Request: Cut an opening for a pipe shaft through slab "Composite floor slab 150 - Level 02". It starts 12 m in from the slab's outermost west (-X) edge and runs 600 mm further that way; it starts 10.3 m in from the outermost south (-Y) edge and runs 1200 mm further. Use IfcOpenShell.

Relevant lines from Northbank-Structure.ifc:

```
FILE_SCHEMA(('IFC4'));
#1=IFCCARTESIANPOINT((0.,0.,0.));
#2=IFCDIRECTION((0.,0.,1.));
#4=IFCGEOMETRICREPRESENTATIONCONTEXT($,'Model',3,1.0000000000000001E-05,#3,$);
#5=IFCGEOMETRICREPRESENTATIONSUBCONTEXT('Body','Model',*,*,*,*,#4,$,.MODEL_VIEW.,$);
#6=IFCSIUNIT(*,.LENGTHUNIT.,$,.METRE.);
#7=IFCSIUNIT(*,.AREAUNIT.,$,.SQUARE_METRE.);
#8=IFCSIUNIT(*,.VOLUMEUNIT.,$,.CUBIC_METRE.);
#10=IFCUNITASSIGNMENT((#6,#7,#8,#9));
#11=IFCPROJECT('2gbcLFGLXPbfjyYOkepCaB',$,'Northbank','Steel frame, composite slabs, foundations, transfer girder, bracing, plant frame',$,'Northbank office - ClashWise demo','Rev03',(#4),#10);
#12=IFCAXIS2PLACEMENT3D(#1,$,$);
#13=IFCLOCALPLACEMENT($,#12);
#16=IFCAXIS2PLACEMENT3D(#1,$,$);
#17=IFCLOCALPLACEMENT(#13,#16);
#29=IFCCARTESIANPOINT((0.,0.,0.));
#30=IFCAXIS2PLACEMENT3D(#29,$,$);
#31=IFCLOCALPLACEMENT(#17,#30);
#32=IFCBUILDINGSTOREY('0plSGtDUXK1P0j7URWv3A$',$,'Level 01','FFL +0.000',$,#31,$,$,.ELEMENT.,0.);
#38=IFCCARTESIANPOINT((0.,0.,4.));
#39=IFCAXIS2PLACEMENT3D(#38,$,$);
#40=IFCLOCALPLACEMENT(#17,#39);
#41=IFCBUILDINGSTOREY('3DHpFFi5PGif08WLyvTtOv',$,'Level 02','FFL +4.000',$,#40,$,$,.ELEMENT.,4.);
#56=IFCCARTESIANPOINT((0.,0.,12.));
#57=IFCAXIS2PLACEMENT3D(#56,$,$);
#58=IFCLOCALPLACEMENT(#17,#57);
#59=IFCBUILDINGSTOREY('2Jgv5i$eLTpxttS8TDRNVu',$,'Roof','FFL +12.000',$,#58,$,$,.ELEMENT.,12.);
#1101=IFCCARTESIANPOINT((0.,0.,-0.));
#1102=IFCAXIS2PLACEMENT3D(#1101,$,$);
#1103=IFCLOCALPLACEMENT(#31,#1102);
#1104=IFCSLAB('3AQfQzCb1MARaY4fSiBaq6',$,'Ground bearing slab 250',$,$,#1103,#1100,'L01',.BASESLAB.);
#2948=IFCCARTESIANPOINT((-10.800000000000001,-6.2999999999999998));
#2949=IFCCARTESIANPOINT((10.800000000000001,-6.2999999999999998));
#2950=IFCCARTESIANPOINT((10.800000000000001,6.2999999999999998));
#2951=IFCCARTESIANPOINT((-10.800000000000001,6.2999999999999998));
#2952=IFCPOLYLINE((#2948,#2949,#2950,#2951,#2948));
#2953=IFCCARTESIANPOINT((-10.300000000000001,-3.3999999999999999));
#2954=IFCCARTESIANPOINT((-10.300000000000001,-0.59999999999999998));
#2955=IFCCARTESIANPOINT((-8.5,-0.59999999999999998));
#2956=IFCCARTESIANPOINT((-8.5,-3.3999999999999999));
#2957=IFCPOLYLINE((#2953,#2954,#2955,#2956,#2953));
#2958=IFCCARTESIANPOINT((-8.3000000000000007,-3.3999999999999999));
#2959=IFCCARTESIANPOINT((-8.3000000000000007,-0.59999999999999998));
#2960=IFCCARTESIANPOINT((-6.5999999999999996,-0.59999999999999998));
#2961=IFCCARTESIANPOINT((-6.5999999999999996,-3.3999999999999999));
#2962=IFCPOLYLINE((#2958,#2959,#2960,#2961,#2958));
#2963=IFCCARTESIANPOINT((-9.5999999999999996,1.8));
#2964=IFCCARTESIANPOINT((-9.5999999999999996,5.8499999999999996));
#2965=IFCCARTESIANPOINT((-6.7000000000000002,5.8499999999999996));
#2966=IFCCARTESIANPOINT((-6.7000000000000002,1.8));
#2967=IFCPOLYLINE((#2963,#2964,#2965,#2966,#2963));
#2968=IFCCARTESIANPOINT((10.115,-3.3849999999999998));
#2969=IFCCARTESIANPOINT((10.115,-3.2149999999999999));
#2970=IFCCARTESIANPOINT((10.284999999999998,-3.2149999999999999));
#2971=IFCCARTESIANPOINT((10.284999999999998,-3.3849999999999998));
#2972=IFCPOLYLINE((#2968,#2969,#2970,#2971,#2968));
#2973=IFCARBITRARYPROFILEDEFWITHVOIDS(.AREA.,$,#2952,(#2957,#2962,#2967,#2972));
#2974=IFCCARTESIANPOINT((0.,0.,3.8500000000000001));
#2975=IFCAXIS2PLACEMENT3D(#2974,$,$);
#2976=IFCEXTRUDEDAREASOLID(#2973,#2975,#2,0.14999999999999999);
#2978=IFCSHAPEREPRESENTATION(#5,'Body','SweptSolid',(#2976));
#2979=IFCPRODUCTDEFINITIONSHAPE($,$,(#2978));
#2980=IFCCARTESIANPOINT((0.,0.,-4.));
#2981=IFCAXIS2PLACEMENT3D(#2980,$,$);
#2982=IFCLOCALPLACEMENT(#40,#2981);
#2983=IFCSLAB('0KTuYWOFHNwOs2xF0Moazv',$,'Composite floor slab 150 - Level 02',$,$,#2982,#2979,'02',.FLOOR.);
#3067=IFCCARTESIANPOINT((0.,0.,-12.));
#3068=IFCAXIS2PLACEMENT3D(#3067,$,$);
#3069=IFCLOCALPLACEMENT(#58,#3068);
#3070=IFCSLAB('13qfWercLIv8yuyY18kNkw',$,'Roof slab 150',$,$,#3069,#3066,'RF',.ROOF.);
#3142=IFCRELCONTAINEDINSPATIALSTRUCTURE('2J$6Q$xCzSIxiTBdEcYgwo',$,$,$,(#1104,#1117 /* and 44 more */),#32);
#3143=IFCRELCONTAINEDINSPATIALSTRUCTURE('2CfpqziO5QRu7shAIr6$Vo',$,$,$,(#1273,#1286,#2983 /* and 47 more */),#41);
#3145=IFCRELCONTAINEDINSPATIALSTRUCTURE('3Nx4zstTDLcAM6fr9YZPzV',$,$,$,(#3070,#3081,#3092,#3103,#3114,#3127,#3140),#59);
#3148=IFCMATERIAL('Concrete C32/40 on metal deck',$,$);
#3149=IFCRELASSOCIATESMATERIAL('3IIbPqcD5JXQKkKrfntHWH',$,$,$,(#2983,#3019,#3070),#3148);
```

```python
import numpy as np
import ifcopenshell
import ifcopenshell.api.feature
import ifcopenshell.api.geometry
import ifcopenshell.api.root
import ifcopenshell.geom
import ifcopenshell.util.placement
import ifcopenshell.util.representation
import ifcopenshell.util.shape
import ifcopenshell.util.unit

model = ifcopenshell.open("Northbank-Structure.ifc")
unit_scale = ifcopenshell.util.unit.calculate_unit_scale(model)
settings = ifcopenshell.geom.settings()


def volume(element):
    """Net volume in cubic metres, openings subtracted."""
    shape = ifcopenshell.geom.create_shape(settings, element)
    return ifcopenshell.util.shape.get_volume(shape.geometry)


slab = model.by_guid("0KTuYWOFHNwOs2xF0Moazv")
before = volume(slab)

# Extent in the slab's own axes, in metres. The edges named are its -X and -Y sides.
slab_shape = ifcopenshell.geom.create_shape(settings, slab)
vertices = ifcopenshell.util.shape.get_vertices(slab_shape.geometry)
x_min, y_min, bottom = vertices.min(axis=0)
top = vertices[:, 2].max()

opening = ifcopenshell.api.root.create_entity(model, ifc_class="IfcOpeningElement", name="Pipe shaft opening", predefined_type="OPENING")
context = ifcopenshell.util.representation.get_context(model, "Model", "Body", "MODEL_VIEW")
width, depth = 0.6, 1.2
outline = [(0.0, 0.0), (width, 0.0), (width, depth), (0.0, depth), (0.0, 0.0)]
# Overshoot both faces by 50 mm so the cut is clean.
shape = ifcopenshell.api.geometry.add_slab_representation(
    model, context=context, depth=top - bottom + 0.1, polyline=outline
)
ifcopenshell.api.geometry.assign_representation(model, product=opening, representation=shape)

matrix = ifcopenshell.util.placement.get_local_placement(slab.ObjectPlacement)
matrix[:, 3] = matrix @ np.append(np.array([x_min + 12, y_min + 10.3, bottom - 0.05]) / unit_scale, 1.0)
ifcopenshell.api.geometry.edit_object_placement(model, product=opening, matrix=matrix, is_si=False)
ifcopenshell.api.feature.add_feature(model, feature=opening, element=slab)

after = volume(slab)

print(f"slab volume {before:.3f} -> {after:.3f} m3")

model.write("Northbank-Structure_rev.ifc")
```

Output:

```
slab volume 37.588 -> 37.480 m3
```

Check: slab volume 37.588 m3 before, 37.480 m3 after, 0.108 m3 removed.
